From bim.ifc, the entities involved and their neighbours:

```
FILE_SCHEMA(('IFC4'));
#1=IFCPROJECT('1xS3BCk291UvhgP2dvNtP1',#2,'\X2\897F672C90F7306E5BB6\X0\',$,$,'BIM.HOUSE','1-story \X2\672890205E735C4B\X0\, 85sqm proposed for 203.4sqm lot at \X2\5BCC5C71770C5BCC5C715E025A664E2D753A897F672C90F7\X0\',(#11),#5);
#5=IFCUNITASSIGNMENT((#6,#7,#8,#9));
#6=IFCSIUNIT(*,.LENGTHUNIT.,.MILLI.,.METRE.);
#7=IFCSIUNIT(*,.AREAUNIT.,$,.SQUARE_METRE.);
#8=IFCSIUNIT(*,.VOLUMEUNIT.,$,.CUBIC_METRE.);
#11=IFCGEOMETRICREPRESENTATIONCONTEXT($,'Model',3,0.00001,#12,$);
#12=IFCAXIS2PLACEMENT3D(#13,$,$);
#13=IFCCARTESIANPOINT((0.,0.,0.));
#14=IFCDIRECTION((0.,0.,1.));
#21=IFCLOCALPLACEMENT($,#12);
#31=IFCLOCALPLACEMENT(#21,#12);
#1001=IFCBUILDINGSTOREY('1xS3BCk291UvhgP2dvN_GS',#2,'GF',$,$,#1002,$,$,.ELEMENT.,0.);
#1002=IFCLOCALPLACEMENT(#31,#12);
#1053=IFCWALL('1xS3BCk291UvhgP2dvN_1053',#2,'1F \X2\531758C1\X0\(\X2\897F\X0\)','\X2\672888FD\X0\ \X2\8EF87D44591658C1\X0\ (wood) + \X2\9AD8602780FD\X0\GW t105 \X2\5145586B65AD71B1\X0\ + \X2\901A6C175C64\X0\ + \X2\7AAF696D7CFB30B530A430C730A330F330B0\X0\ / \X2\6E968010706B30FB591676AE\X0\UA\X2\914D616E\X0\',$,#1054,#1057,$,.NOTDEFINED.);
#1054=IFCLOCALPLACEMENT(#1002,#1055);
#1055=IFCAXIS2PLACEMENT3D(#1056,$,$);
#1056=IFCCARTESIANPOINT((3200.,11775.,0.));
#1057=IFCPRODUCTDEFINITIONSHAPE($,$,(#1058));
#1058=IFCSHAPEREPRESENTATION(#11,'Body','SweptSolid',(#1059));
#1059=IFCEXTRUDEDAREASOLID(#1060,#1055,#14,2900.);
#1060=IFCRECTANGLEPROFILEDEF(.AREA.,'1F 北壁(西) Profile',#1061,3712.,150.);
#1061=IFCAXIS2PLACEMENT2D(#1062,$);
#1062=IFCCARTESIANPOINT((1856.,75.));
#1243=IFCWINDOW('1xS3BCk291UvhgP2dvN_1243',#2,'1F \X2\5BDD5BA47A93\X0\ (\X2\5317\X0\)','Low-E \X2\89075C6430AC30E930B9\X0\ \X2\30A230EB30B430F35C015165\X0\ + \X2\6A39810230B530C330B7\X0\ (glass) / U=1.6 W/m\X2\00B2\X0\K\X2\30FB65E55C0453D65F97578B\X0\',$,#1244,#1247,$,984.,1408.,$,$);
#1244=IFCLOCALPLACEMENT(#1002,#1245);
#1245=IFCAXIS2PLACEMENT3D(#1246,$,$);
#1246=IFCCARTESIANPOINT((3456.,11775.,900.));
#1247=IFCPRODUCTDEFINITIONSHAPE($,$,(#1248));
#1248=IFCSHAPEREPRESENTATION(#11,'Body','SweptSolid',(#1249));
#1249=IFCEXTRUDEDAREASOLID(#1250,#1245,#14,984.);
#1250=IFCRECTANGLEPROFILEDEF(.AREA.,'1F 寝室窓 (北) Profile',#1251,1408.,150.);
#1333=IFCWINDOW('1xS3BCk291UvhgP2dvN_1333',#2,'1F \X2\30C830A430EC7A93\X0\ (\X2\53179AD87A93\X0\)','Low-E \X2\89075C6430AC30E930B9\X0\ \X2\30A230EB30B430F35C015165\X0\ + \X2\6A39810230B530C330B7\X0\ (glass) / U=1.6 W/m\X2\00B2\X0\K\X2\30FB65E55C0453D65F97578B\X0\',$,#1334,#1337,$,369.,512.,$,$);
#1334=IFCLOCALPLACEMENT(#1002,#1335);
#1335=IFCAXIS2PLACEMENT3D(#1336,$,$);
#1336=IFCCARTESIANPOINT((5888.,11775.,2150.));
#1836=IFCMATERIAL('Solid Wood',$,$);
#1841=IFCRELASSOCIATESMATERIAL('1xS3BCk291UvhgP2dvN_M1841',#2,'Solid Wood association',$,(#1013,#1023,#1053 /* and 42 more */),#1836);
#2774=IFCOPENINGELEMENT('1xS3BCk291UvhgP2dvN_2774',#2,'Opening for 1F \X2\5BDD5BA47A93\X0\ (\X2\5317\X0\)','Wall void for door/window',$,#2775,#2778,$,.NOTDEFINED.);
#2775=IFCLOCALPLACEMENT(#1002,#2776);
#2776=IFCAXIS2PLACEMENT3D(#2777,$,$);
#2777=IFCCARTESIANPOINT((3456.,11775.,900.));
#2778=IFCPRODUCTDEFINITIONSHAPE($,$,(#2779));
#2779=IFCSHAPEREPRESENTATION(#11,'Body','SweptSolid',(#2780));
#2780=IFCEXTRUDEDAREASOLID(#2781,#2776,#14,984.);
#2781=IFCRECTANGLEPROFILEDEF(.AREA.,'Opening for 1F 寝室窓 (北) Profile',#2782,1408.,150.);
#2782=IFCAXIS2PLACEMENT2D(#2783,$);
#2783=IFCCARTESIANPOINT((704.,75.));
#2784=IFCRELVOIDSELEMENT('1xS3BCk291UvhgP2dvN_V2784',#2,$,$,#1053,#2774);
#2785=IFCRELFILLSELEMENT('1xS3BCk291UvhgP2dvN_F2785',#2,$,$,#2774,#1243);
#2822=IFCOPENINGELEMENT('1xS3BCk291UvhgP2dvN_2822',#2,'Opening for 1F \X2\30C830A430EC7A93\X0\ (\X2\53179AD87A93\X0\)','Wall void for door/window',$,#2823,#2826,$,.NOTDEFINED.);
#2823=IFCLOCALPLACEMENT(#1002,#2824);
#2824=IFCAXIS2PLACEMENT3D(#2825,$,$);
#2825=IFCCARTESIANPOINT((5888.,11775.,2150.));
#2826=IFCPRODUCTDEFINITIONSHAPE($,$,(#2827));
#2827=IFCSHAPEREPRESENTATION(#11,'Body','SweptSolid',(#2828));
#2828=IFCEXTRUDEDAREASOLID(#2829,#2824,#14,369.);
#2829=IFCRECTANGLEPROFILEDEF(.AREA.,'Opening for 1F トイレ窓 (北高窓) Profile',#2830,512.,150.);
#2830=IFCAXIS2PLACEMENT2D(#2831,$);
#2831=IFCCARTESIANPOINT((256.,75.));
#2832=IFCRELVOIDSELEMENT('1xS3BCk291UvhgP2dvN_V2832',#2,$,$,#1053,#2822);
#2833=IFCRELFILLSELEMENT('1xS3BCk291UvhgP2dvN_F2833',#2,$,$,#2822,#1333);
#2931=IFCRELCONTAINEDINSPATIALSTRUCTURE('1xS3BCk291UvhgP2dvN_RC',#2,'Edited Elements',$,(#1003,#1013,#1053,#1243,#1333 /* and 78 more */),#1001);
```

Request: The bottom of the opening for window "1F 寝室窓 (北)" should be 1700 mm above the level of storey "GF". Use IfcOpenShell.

```python
import numpy as np
import ifcopenshell
import ifcopenshell.api.geometry
import ifcopenshell.geom
import ifcopenshell.util.element
import ifcopenshell.util.placement
import ifcopenshell.util.shape
import ifcopenshell.util.unit

model = ifcopenshell.open("bim.ifc")
unit_scale = ifcopenshell.util.unit.calculate_unit_scale(model)

window = model.by_guid("1xS3BCk291UvhgP2dvN_1243")
opening = window.FillsVoids[0].RelatingOpeningElement
storey = ifcopenshell.util.element.get_container(window, ifc_class="IfcBuildingStorey")
level = ifcopenshell.util.placement.get_local_placement(storey.ObjectPlacement)[2, 3]

# The opening's origin need not be at the sill, so measure its lowest point.
shape = ifcopenshell.geom.create_shape(ifcopenshell.geom.settings(), opening)
bottom = ifcopenshell.util.shape.get_shape_bottom_elevation(shape, shape.geometry) / unit_scale
dz = level + 1.7 / unit_scale - bottom

shift = np.array([0.0, 0.0, dz])
# The window is not placed relative to its opening, so move both.
for product in (opening, window):
    matrix = ifcopenshell.util.placement.get_local_placement(product.ObjectPlacement)
    matrix[:3, 3] += shift
    ifcopenshell.api.geometry.edit_object_placement(model, product=product, matrix=matrix, is_si=False)

print(f"moved by {dz * unit_scale:+.3f} m")

model.write("bim_updated.ifc")
```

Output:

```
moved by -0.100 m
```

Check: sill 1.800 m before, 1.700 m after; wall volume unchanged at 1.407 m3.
